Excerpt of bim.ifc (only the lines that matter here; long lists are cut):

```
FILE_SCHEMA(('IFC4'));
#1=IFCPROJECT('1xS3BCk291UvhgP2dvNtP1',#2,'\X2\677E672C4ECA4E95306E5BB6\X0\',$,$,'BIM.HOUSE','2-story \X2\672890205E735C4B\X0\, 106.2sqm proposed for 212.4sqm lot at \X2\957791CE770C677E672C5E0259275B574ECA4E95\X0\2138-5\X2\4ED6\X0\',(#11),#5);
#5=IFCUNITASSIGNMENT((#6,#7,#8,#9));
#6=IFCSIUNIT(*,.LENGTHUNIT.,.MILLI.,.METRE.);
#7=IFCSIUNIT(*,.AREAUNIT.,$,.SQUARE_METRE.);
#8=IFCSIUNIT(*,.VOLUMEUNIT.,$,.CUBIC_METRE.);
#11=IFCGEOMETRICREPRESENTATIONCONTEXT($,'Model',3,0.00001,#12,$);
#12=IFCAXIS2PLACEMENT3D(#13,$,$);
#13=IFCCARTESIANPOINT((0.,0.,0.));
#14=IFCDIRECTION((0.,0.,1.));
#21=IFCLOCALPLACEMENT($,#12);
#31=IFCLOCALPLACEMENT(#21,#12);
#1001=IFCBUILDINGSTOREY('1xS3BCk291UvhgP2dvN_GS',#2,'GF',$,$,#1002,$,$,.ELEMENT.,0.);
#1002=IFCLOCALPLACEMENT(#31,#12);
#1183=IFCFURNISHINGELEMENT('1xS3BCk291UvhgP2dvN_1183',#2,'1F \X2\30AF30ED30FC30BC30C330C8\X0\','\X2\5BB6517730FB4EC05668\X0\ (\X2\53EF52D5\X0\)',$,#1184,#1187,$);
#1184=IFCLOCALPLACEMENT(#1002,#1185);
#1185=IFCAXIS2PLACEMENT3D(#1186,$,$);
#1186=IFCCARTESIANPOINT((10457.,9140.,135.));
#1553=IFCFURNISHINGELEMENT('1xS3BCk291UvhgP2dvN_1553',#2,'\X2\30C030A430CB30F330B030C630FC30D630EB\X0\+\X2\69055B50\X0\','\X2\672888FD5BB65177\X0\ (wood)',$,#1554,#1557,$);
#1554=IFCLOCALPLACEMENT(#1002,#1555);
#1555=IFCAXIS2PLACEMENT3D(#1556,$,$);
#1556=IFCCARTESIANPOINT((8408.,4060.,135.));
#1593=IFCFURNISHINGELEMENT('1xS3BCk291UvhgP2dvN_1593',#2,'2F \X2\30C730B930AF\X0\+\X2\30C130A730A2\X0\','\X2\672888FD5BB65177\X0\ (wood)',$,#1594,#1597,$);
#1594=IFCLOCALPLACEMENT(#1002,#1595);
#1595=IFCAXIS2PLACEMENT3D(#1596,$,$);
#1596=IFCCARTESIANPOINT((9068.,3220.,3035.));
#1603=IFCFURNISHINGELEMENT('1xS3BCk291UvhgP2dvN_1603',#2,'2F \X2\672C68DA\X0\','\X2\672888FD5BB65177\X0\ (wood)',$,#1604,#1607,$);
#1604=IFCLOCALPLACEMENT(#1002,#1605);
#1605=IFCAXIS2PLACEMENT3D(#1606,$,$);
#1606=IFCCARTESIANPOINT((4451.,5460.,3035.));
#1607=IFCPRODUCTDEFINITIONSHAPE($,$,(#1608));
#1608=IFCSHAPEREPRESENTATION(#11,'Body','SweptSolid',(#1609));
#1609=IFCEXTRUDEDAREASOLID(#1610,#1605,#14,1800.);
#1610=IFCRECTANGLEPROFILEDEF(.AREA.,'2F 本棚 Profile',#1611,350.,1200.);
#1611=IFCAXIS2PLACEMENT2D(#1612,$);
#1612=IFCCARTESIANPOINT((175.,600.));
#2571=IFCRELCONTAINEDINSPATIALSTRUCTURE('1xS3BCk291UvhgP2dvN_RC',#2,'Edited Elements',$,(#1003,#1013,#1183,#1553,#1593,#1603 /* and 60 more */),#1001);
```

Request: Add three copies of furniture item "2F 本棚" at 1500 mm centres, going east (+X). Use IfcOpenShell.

```python
import numpy as np
import ifcopenshell
import ifcopenshell.api.geometry
import ifcopenshell.api.root
import ifcopenshell.util.element
import ifcopenshell.util.placement
import ifcopenshell.util.unit

model = ifcopenshell.open("bim.ifc")
unit_scale = ifcopenshell.util.unit.calculate_unit_scale(model)


def reuse_history(source, copy):
    """copy_class also copies each property set's owner history, people and application; keep the originals."""
    for rel in copy.IsDefinedBy:
        if rel.is_a("IfcRelDefinesByProperties") and (history := rel.RelatingPropertyDefinition.OwnerHistory):
            rel.RelatingPropertyDefinition.OwnerHistory = source.OwnerHistory
            ifcopenshell.util.element.remove_deep2(model, history)


source = model.by_id(1603)
base = ifcopenshell.util.placement.get_local_placement(source.ObjectPlacement)
step = np.array([1.0, 0.0, 0.0]) * 1.5 / unit_scale

for i in range(1, 4):
    copy = ifcopenshell.api.root.copy_class(model, product=source)
    copy.Representation = ifcopenshell.util.element.copy_deep(
        model, source.Representation, exclude=["IfcGeometricRepresentationContext", "IfcRepresentationMap"]
    )
    reuse_history(source, copy)
    matrix = base.copy()
    matrix[:3, 3] += i * step
    print("added at", matrix[:3, 3].round(3) + 0.0)
    ifcopenshell.api.geometry.edit_object_placement(model, product=copy, matrix=matrix, is_si=False)

model.write("bim_rev.ifc")
```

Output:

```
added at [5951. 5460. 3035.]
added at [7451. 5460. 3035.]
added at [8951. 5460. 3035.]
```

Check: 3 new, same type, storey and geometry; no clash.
